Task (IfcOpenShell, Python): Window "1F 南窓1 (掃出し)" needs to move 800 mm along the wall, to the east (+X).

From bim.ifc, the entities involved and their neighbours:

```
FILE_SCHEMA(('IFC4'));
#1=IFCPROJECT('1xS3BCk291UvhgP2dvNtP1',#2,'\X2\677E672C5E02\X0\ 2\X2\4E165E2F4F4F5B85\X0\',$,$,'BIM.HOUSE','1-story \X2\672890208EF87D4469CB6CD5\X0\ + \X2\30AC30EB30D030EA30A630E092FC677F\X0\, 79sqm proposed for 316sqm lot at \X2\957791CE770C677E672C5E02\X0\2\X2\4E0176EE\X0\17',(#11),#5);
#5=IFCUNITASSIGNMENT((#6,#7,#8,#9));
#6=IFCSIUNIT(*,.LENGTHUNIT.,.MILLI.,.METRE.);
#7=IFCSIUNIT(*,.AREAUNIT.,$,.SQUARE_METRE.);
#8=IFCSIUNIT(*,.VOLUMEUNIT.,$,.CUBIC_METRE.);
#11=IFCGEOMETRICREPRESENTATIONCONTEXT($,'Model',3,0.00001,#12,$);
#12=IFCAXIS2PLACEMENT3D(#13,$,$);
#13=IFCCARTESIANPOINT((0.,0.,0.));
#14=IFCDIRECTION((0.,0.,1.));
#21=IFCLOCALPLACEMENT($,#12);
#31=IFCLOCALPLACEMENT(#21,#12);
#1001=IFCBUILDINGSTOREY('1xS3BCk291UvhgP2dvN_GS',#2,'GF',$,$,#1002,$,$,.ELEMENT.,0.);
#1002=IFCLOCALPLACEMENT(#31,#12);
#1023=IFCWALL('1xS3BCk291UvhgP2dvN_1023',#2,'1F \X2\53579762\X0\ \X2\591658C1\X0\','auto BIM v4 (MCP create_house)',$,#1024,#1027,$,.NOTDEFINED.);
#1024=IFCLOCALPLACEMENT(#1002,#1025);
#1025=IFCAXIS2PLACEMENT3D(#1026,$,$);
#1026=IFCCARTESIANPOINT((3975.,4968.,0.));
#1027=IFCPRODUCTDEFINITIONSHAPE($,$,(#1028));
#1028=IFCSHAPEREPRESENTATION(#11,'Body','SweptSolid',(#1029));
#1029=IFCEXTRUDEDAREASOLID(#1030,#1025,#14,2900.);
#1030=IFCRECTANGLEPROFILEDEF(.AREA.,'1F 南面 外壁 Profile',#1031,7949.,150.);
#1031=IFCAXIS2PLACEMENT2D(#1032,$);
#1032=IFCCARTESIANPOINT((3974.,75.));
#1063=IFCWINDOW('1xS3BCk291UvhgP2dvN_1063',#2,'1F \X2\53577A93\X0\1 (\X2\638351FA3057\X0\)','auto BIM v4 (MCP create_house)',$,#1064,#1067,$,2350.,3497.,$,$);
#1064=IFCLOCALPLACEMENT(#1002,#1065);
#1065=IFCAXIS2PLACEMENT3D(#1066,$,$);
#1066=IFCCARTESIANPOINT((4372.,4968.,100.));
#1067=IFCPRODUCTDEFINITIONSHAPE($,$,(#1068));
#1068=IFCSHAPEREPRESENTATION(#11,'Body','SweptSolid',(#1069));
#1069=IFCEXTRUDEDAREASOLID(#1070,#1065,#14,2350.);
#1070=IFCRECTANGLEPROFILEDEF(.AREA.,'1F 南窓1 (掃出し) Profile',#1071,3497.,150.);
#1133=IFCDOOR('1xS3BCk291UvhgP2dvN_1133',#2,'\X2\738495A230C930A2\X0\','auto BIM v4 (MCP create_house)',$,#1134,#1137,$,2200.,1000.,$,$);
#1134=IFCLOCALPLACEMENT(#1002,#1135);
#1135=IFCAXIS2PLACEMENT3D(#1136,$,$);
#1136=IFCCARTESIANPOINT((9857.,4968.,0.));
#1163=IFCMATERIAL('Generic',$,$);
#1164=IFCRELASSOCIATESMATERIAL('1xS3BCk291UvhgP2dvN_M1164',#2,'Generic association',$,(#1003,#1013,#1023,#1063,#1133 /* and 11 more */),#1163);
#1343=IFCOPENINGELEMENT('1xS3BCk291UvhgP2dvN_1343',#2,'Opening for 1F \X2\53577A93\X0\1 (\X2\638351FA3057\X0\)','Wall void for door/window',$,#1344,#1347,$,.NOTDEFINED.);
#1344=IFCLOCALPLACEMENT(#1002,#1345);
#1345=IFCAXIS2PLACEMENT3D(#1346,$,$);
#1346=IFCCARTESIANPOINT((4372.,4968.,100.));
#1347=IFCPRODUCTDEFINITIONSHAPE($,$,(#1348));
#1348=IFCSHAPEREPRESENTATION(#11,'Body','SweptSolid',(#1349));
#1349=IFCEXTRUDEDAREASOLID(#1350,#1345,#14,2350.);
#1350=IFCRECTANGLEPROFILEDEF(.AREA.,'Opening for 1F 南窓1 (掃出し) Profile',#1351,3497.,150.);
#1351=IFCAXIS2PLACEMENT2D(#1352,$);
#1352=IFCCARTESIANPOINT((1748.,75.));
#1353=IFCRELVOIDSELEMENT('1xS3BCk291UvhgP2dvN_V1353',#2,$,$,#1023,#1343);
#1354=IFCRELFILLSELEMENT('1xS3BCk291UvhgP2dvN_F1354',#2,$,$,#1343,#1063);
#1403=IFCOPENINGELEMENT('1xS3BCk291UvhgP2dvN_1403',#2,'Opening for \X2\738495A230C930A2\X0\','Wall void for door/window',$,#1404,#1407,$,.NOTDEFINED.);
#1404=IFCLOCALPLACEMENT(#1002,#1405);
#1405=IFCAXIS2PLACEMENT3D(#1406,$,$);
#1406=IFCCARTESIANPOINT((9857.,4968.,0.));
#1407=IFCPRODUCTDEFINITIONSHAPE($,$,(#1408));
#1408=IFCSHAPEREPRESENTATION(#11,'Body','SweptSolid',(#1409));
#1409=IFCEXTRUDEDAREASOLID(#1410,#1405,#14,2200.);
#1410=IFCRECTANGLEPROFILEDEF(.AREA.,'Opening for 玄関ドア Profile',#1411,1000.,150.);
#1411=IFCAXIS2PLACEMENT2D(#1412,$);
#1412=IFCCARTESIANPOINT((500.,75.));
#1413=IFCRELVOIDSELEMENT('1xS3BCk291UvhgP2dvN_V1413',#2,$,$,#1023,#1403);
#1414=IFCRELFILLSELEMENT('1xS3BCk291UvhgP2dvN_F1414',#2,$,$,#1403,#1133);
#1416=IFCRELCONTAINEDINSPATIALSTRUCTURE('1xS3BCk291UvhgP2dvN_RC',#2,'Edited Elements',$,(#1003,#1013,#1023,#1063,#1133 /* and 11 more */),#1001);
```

```python
import ifcopenshell
import ifcopenshell.api.geometry
import ifcopenshell.util.placement

model = ifcopenshell.open("bim.ifc")

window = model.by_guid("1xS3BCk291UvhgP2dvN_1063")
opening = window.FillsVoids[0].RelatingOpeningElement
wall = opening.VoidsElements[0].RelatingBuildingElement

wall_matrix = ifcopenshell.util.placement.get_local_placement(wall.ObjectPlacement)
shift = wall_matrix[:3, 0] * 800.0
before = ifcopenshell.util.placement.get_local_placement(window.ObjectPlacement)[:3, 3].copy()

# The window is not placed relative to its opening, so move both.
for product in (opening, window):
    matrix = ifcopenshell.util.placement.get_local_placement(product.ObjectPlacement)
    matrix[:3, 3] += shift
    ifcopenshell.api.geometry.edit_object_placement(model, product=product, matrix=matrix, is_si=False)

after = ifcopenshell.util.placement.get_local_placement(window.ObjectPlacement)[:3, 3]
print("window moved by", (after - before).round(3) + 0.0)

model.write("bim_edited.ifc")
```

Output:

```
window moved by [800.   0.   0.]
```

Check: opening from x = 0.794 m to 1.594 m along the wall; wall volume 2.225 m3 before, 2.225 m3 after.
